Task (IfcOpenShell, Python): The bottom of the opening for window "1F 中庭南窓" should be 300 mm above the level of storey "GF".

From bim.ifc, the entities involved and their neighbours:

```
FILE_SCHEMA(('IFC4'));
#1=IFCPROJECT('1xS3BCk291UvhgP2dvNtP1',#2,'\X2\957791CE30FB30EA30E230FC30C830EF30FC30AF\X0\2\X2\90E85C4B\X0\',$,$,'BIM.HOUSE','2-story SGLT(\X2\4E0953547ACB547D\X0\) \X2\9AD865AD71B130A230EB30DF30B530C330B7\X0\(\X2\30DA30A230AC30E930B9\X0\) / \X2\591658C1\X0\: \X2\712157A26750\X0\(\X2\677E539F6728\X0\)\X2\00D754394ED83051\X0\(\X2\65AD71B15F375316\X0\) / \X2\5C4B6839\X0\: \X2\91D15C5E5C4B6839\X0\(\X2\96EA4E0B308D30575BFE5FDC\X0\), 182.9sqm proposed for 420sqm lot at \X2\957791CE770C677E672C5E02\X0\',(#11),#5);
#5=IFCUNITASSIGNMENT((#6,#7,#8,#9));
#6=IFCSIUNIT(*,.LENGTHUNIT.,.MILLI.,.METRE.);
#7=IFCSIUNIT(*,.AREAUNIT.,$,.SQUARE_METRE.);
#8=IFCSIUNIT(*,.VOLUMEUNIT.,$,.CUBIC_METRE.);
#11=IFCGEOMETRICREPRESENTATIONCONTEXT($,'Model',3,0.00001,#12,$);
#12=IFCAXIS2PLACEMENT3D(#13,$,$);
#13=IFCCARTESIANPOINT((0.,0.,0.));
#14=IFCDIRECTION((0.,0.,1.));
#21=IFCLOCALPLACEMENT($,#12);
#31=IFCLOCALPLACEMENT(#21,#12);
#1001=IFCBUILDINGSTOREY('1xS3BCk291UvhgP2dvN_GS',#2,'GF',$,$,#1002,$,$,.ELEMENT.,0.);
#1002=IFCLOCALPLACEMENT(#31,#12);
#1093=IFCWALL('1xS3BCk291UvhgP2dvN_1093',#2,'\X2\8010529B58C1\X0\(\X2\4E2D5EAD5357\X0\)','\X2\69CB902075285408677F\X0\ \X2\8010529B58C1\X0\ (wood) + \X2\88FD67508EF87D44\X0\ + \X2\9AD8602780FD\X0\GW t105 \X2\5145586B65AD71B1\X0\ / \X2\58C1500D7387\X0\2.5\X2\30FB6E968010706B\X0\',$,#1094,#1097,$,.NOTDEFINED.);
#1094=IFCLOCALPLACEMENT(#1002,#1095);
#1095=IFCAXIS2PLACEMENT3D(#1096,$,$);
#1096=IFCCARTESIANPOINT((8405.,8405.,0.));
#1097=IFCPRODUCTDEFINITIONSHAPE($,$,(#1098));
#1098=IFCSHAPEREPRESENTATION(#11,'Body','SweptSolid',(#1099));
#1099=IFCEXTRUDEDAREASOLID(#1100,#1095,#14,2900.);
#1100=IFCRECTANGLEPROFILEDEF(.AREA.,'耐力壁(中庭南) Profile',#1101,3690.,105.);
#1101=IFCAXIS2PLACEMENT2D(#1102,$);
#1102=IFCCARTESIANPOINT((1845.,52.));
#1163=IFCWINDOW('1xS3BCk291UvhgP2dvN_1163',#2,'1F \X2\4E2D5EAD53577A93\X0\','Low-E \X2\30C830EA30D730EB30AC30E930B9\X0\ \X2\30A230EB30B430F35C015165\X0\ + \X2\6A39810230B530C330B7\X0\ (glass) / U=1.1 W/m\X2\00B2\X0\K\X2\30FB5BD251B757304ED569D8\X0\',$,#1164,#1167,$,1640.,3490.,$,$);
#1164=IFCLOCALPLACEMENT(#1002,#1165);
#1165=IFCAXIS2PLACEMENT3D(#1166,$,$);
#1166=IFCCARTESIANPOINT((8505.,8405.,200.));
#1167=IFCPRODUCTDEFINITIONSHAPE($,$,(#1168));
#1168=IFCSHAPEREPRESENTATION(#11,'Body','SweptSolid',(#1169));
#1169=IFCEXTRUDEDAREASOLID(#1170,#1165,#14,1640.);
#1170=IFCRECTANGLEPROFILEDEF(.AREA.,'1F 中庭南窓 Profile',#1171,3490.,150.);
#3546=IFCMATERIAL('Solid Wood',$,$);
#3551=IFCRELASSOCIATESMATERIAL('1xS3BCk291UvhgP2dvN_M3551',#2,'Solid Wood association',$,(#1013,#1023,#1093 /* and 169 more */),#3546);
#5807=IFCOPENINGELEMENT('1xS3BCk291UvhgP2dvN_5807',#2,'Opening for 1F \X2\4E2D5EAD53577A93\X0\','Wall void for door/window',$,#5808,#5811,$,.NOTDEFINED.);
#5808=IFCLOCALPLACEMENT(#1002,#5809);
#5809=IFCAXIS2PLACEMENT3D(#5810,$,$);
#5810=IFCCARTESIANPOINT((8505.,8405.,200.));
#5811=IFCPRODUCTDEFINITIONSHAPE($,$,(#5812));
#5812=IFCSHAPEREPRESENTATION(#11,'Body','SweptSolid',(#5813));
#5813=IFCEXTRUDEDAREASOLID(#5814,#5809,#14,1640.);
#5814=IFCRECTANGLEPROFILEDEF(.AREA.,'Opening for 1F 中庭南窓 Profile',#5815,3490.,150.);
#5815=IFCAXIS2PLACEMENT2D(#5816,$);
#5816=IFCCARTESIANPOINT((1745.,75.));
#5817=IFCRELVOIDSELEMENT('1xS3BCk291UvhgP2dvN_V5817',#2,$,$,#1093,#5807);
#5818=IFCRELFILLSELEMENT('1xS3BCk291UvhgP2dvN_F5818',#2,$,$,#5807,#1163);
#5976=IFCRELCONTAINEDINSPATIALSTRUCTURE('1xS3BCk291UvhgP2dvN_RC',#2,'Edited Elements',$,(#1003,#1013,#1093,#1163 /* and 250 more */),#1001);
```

```python
import numpy as np
import ifcopenshell
import ifcopenshell.api.geometry
import ifcopenshell.geom
import ifcopenshell.util.element
import ifcopenshell.util.placement
import ifcopenshell.util.shape
import ifcopenshell.util.unit

model = ifcopenshell.open("bim.ifc")
unit_scale = ifcopenshell.util.unit.calculate_unit_scale(model)

window = model.by_guid("1xS3BCk291UvhgP2dvN_1163")
opening = window.FillsVoids[0].RelatingOpeningElement
storey = ifcopenshell.util.element.get_container(window, ifc_class="IfcBuildingStorey")
level = ifcopenshell.util.placement.get_local_placement(storey.ObjectPlacement)[2, 3]

# The opening's origin need not be at the sill, so measure its lowest point.
shape = ifcopenshell.geom.create_shape(ifcopenshell.geom.settings(), opening)
bottom = ifcopenshell.util.shape.get_shape_bottom_elevation(shape, shape.geometry) / unit_scale
dz = level + 0.3 / unit_scale - bottom

shift = np.array([0.0, 0.0, dz])
# The window is not placed relative to its opening, so move both.
for product in (opening, window):
    matrix = ifcopenshell.util.placement.get_local_placement(product.ObjectPlacement)
    matrix[:3, 3] += shift
    ifcopenshell.api.geometry.edit_object_placement(model, product=product, matrix=matrix, is_si=False)

print(f"moved by {dz * unit_scale:+.3f} m")

model.write("bim_rev.ifc")
```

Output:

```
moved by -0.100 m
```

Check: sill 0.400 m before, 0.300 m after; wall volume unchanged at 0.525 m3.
